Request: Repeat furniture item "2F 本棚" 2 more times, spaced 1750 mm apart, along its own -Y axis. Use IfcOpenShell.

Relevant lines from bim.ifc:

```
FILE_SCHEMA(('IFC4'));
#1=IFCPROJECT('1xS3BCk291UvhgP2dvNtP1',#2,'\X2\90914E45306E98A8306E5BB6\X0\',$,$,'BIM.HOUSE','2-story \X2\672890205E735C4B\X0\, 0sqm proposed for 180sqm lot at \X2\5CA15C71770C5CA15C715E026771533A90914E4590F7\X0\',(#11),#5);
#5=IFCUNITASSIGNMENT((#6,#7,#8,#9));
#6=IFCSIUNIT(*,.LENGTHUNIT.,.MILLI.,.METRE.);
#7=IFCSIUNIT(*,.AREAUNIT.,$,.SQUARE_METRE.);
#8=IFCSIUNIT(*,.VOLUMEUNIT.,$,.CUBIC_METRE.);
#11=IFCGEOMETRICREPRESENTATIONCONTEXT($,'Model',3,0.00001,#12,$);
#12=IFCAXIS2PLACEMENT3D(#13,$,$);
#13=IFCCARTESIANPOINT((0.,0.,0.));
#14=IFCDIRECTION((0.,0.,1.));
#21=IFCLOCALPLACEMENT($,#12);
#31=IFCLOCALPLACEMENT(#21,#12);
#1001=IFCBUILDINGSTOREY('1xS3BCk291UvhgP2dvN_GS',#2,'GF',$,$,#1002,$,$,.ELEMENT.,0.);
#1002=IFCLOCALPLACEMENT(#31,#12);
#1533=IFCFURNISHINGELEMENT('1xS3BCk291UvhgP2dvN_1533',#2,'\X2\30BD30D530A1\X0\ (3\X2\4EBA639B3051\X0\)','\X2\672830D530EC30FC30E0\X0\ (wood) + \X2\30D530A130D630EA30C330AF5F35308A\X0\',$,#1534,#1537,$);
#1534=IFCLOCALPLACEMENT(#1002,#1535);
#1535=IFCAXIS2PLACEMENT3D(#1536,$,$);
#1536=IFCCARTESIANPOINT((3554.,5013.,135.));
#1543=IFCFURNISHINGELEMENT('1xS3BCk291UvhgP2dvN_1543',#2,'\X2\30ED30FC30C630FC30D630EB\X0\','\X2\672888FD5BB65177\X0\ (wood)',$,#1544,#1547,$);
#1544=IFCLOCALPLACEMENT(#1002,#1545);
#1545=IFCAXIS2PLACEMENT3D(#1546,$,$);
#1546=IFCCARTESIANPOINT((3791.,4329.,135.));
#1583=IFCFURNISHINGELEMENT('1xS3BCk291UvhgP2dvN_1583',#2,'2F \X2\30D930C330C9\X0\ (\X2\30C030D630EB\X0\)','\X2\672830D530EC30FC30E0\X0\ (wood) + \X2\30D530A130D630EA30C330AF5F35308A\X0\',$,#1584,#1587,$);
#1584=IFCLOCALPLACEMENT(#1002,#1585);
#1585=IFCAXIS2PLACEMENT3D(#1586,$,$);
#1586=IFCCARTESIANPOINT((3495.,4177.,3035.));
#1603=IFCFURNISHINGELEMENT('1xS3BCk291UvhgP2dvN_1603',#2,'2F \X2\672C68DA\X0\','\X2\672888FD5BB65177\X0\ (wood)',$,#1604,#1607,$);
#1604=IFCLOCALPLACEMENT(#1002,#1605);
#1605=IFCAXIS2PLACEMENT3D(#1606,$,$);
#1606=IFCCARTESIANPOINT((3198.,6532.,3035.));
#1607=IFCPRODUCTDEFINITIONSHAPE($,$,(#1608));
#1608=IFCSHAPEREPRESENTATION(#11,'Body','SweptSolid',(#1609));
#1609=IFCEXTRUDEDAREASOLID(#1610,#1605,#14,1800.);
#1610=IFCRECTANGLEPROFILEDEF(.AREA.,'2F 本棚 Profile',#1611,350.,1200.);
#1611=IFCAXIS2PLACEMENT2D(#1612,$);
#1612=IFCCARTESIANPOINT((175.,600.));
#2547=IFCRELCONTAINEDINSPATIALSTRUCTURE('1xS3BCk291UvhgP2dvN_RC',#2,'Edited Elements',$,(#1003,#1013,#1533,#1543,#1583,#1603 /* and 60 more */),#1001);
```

```python
import ifcopenshell
import ifcopenshell.api.geometry
import ifcopenshell.api.root
import ifcopenshell.util.element
import ifcopenshell.util.placement
import ifcopenshell.util.unit

model = ifcopenshell.open("bim.ifc")
unit_scale = ifcopenshell.util.unit.calculate_unit_scale(model)


def reuse_history(source, copy):
    """copy_class also copies each property set's owner history, people and application; keep the originals."""
    for rel in copy.IsDefinedBy:
        if rel.is_a("IfcRelDefinesByProperties") and (history := rel.RelatingPropertyDefinition.OwnerHistory):
            rel.RelatingPropertyDefinition.OwnerHistory = source.OwnerHistory
            ifcopenshell.util.element.remove_deep2(model, history)


source = model.by_id(1603)
base = ifcopenshell.util.placement.get_local_placement(source.ObjectPlacement)
step = -base[:3, 1] * 1.75 / unit_scale

for i in range(1, 3):
    copy = ifcopenshell.api.root.copy_class(model, product=source)
    copy.Representation = ifcopenshell.util.element.copy_deep(
        model, source.Representation, exclude=["IfcGeometricRepresentationContext", "IfcRepresentationMap"]
    )
    reuse_history(source, copy)
    matrix = base.copy()
    matrix[:3, 3] += i * step
    print("added at", matrix[:3, 3].round(3) + 0.0)
    ifcopenshell.api.geometry.edit_object_placement(model, product=copy, matrix=matrix, is_si=False)

model.write("bim-out.ifc")
```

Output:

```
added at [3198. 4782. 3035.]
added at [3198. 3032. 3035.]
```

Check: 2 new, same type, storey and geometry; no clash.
